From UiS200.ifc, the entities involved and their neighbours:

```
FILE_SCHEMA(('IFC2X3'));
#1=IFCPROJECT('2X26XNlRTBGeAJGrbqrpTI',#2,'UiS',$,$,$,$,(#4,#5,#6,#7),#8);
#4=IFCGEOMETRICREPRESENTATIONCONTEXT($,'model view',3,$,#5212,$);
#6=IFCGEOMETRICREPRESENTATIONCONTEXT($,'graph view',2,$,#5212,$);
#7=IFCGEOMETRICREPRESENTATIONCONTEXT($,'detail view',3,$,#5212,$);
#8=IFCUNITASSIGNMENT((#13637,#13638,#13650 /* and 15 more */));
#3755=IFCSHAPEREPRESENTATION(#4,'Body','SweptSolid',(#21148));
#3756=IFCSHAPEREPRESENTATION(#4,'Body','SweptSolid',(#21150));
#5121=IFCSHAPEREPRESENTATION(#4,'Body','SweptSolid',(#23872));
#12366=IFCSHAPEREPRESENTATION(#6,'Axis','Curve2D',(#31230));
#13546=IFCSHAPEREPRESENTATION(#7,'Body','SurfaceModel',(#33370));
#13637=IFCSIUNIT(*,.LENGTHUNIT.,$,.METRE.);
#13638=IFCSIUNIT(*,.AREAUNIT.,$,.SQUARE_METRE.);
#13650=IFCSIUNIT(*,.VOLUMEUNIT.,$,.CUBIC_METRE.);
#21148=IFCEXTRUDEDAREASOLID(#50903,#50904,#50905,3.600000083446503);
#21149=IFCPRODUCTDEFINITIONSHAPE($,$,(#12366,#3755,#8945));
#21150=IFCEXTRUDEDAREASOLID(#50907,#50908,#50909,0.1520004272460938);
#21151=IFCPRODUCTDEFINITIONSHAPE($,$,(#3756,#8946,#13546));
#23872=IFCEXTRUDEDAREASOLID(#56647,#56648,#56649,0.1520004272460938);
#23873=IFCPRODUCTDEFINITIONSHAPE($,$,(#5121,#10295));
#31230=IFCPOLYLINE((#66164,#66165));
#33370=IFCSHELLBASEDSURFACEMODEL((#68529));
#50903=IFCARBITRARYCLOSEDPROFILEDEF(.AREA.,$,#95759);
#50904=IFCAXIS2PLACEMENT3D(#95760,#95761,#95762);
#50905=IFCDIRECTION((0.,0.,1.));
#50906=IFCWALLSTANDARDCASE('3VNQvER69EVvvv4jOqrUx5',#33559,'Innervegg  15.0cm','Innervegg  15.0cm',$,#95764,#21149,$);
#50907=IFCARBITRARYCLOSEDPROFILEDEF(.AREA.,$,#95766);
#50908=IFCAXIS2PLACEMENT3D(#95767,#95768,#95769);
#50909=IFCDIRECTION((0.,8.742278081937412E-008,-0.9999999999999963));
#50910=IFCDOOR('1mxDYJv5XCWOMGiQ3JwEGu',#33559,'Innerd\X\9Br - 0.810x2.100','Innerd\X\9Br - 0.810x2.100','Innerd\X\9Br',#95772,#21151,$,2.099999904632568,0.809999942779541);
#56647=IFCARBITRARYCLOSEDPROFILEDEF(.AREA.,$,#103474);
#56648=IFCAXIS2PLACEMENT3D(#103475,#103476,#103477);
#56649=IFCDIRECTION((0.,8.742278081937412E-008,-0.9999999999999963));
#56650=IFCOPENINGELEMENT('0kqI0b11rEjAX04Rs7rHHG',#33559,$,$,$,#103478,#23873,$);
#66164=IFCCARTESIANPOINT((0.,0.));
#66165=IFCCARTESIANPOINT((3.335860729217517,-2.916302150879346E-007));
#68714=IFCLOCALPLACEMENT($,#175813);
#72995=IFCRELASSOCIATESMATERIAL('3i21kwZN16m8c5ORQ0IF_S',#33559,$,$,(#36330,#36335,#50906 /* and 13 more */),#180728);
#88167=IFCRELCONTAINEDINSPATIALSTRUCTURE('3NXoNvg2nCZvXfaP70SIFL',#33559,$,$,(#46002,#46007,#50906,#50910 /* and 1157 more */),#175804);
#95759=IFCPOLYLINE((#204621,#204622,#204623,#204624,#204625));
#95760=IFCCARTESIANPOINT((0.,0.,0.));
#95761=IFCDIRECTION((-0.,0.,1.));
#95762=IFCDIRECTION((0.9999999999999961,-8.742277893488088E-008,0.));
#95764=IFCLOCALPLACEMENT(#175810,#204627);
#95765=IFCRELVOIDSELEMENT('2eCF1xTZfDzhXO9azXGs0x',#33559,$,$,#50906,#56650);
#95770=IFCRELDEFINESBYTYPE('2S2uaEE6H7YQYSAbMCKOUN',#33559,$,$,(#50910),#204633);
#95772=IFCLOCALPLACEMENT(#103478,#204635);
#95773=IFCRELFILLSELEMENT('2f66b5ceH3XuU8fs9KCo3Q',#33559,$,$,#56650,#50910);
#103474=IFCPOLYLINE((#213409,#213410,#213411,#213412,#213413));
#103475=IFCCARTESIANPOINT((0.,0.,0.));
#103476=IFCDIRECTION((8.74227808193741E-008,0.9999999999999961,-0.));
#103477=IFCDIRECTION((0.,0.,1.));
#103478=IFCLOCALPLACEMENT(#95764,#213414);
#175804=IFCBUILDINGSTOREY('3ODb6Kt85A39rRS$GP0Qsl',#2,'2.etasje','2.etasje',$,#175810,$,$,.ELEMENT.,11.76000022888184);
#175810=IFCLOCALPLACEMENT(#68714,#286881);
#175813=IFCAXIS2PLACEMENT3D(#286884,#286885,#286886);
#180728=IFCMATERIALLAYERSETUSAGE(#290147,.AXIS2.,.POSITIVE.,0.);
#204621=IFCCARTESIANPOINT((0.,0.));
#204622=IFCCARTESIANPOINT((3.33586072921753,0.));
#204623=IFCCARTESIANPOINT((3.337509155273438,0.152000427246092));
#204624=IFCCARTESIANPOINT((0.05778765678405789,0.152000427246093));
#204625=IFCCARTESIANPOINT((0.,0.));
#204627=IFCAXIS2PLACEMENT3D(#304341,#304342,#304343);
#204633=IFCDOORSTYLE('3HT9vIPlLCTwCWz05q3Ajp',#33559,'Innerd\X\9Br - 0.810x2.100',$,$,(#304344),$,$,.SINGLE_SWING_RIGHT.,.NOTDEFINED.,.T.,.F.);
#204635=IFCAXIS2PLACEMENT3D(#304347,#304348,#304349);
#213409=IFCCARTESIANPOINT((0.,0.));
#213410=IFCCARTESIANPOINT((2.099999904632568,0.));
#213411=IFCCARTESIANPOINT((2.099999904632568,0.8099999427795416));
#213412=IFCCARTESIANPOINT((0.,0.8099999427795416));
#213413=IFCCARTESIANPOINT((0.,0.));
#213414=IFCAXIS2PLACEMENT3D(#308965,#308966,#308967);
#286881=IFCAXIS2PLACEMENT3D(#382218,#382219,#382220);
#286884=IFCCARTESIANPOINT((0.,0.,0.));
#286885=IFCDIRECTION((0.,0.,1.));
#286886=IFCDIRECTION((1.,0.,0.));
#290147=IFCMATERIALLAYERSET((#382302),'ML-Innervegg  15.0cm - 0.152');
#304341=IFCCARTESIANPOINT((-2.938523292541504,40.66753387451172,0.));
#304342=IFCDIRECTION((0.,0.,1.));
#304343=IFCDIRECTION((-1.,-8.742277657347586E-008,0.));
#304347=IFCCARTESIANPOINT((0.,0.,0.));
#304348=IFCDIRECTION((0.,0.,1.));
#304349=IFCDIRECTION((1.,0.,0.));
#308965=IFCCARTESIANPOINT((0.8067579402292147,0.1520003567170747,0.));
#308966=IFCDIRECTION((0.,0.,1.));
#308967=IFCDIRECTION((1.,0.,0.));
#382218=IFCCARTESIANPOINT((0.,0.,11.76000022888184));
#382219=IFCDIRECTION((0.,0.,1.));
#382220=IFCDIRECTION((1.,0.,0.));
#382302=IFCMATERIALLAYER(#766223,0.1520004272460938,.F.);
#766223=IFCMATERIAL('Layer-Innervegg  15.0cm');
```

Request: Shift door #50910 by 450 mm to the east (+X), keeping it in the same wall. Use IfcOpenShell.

```python
import ifcopenshell
import ifcopenshell.api.geometry
import ifcopenshell.util.placement

model = ifcopenshell.open("UiS200.ifc")

door = model.by_id(50910)
opening = door.FillsVoids[0].RelatingOpeningElement
wall = opening.VoidsElements[0].RelatingBuildingElement

wall_matrix = ifcopenshell.util.placement.get_local_placement(wall.ObjectPlacement)
shift = wall_matrix[:3, 0] * -0.45
before = ifcopenshell.util.placement.get_local_placement(door.ObjectPlacement)[:3, 3].copy()

# The door is placed relative to its opening, so it follows when the opening moves.
matrix = ifcopenshell.util.placement.get_local_placement(opening.ObjectPlacement)
matrix[:3, 3] += shift
ifcopenshell.api.geometry.edit_object_placement(
    model, product=opening, matrix=matrix, is_si=False, should_transform_children=True
)

after = ifcopenshell.util.placement.get_local_placement(door.ObjectPlacement)[:3, 3]
print("door moved by", (after - before).round(3) + 0.0)

model.write("UiS200-out.ifc")
```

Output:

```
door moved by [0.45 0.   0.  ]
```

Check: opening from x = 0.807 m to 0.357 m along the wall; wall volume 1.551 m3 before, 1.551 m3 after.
